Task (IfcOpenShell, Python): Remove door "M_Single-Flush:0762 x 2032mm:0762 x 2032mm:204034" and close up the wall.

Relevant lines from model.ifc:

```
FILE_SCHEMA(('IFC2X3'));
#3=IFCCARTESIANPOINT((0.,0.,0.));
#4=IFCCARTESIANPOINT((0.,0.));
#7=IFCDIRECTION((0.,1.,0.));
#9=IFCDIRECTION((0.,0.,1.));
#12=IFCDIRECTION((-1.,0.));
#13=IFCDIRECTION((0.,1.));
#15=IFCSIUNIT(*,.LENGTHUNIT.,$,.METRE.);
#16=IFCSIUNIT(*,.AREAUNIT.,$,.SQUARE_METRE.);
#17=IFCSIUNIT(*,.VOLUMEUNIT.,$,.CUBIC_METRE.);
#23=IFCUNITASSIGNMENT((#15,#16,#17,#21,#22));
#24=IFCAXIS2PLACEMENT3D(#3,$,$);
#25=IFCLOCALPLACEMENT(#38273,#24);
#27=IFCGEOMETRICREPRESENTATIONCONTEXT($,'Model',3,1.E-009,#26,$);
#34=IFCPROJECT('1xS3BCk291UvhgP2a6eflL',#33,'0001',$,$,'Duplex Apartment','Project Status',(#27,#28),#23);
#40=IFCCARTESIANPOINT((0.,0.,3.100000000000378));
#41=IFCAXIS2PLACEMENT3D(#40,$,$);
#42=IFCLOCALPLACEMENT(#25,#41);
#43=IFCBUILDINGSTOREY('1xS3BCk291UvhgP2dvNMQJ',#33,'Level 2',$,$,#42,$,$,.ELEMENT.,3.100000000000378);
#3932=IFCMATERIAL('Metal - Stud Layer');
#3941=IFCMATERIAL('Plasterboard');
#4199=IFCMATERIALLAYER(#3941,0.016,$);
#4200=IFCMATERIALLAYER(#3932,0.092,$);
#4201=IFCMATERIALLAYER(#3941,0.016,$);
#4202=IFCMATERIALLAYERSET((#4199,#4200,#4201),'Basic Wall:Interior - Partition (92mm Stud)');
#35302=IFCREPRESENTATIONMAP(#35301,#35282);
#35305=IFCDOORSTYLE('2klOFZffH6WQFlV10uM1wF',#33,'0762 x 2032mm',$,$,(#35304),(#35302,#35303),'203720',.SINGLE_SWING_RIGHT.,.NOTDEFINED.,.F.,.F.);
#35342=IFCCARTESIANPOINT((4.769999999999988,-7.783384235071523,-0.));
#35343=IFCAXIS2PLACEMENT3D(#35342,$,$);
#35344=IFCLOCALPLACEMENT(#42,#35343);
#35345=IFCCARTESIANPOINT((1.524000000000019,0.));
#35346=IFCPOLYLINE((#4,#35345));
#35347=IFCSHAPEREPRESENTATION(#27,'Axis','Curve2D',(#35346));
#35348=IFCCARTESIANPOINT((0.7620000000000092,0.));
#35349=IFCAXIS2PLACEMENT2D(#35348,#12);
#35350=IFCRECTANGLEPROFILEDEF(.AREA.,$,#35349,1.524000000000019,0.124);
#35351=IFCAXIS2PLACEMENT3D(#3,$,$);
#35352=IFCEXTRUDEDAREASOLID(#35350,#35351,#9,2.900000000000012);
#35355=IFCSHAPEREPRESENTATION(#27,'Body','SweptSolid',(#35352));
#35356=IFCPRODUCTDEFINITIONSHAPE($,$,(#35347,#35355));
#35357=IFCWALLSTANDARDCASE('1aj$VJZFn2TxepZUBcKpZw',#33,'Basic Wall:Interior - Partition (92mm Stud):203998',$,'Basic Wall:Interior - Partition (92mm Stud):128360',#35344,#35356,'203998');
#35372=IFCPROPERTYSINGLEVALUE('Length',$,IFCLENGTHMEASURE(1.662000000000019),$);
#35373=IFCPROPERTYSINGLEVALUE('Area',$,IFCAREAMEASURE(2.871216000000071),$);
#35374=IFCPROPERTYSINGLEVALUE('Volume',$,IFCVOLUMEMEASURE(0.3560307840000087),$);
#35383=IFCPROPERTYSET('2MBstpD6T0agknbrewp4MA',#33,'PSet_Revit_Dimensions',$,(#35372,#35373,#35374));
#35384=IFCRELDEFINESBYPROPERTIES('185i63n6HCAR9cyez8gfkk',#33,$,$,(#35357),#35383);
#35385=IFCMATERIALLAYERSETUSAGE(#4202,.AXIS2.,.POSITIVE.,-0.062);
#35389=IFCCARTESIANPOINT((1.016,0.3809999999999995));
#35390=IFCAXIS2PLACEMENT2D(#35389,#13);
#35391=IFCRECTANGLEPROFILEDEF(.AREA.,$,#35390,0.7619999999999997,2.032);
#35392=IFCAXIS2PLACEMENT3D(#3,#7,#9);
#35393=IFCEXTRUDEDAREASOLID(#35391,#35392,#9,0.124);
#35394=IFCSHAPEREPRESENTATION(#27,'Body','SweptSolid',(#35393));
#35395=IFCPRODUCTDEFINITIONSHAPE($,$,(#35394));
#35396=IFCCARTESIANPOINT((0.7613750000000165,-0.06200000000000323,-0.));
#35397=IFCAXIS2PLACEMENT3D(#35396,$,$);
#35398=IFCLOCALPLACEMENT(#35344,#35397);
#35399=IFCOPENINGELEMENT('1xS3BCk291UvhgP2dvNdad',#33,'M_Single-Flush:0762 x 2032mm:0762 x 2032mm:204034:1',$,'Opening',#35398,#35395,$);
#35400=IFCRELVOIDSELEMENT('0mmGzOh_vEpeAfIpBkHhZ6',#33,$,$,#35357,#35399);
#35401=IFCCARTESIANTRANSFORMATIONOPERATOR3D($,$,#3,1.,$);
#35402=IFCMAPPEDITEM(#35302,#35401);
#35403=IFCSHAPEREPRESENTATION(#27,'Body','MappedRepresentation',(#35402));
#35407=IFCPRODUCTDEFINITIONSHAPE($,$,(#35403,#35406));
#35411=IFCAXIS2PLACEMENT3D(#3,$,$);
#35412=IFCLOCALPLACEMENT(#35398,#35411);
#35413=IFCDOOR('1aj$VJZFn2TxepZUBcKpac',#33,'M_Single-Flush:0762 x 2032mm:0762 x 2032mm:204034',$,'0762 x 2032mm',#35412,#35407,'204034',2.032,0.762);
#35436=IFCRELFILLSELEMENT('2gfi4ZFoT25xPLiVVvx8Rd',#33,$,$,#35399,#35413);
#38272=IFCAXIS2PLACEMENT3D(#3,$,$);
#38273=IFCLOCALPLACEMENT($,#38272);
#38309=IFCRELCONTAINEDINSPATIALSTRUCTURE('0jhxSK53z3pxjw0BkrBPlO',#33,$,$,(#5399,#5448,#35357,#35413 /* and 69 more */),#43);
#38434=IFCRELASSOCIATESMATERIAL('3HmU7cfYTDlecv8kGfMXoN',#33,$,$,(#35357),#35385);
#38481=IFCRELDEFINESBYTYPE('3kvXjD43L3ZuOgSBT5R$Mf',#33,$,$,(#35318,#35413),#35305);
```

```python
import ifcopenshell
import ifcopenshell.api.feature
import ifcopenshell.api.pset
import ifcopenshell.api.root
import ifcopenshell.geom
import ifcopenshell.util.element
import ifcopenshell.util.shape
import ifcopenshell.util.unit

model = ifcopenshell.open("model.ifc")
area_scale = ifcopenshell.util.unit.calculate_unit_scale(model, "AREAUNIT")
volume_scale = ifcopenshell.util.unit.calculate_unit_scale(model, "VOLUMEUNIT")
settings = ifcopenshell.geom.settings()


def volume(element):
    """Net volume in cubic metres, openings subtracted."""
    shape = ifcopenshell.geom.create_shape(settings, element)
    return ifcopenshell.util.shape.get_volume(shape.geometry)


door = model.by_id(35413)
opening = door.FillsVoids[0].RelatingOpeningElement
wall = opening.VoidsElements[0].RelatingBuildingElement
before = volume(wall)

ifcopenshell.api.root.remove_product(model, product=door)
ifcopenshell.api.feature.remove_feature(model, feature=opening)

after = volume(wall)
thickness = 0.124  # wall thickness in metres

# Update the wall's stored quantities.
pset = model.by_id(ifcopenshell.util.element.get_pset(wall, "PSet_Revit_Dimensions", should_inherit=False)["id"])
ifcopenshell.api.pset.edit_pset(model, pset=pset, properties={
    "Area": model.create_entity("IfcAreaMeasure", after / thickness / area_scale),
    "Volume": model.create_entity("IfcVolumeMeasure", after / volume_scale),
})

print(f"wall volume {before:.3f} -> {after:.3f} m3")

model.write("model-out.ifc")
```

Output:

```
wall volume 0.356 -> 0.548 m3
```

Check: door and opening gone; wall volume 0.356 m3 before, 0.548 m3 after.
